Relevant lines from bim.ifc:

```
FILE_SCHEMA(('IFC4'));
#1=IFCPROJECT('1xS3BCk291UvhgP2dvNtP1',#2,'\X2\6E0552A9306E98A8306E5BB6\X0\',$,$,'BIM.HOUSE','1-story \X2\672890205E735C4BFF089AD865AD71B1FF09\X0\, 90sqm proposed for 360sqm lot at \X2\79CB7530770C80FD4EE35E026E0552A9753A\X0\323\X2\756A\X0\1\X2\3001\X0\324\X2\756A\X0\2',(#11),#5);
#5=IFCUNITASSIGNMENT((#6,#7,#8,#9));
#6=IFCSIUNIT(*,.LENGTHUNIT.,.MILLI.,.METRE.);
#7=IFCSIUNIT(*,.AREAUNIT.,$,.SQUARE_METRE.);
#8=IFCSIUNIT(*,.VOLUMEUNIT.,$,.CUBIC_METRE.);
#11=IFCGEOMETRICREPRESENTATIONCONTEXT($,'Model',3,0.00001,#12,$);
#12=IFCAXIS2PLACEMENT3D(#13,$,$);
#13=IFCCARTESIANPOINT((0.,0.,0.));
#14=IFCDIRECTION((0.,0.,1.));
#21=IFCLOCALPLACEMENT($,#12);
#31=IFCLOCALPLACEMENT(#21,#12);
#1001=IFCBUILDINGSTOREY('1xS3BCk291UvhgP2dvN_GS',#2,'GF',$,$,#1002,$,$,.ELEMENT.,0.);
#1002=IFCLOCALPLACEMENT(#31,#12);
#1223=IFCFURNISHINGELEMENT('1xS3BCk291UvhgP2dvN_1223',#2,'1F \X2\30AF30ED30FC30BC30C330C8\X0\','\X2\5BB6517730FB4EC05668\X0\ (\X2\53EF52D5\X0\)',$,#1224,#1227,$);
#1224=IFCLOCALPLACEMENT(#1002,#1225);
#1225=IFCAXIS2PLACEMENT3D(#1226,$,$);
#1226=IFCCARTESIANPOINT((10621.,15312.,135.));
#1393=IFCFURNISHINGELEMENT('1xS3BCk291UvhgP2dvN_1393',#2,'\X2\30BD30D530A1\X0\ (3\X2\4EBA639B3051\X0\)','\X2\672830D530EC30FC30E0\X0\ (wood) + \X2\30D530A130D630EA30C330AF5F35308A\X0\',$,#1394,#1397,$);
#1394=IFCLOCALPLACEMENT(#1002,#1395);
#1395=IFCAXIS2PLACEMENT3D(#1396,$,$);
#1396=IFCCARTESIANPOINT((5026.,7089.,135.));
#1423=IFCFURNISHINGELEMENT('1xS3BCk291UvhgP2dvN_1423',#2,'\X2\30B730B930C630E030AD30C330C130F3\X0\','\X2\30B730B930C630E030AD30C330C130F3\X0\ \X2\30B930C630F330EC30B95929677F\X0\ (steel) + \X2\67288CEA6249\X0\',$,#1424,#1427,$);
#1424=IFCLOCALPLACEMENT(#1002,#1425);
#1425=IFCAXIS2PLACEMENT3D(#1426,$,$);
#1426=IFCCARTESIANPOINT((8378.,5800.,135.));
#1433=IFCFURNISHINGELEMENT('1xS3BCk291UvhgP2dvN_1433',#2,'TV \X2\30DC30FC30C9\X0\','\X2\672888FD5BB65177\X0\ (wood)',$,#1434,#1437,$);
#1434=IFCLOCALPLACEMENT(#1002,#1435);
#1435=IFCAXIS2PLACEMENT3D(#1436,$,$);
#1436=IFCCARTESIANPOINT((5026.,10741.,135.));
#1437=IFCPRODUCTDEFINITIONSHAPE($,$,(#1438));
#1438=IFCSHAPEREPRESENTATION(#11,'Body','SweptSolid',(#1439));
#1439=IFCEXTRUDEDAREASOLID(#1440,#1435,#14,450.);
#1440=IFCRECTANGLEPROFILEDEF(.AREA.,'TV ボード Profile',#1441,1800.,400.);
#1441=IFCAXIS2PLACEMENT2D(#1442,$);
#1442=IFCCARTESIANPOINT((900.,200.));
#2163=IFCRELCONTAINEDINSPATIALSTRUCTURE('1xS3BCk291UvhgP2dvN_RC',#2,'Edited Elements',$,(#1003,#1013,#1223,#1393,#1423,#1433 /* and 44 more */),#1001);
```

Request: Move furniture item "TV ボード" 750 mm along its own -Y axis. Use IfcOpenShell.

```python
import ifcopenshell
import ifcopenshell.api.geometry
import ifcopenshell.util.placement
import ifcopenshell.util.unit

model = ifcopenshell.open("bim.ifc")
unit_scale = ifcopenshell.util.unit.calculate_unit_scale(model)

item = model.by_id(1433)
matrix = ifcopenshell.util.placement.get_local_placement(item.ObjectPlacement)
matrix[:3, 3] -= matrix[:3, 1] * 0.75 / unit_scale
ifcopenshell.api.geometry.edit_object_placement(model, product=item, matrix=matrix, is_si=False)

print(ifcopenshell.util.placement.get_local_placement(item.ObjectPlacement).round(3) + 0.0)

model.write("bim-out.ifc")
```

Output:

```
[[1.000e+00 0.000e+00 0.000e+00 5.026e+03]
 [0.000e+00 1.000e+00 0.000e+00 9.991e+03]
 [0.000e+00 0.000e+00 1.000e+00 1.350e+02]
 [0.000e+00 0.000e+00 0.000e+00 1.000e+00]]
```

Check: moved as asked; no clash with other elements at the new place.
